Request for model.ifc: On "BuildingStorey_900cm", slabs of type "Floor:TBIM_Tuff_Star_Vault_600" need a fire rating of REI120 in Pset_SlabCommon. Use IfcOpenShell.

First a look at what the model holds.

```python
import ifcopenshell
import ifcopenshell.util.element

model = ifcopenshell.open("model.ifc")
print(model.schema)
storey = next(s for s in model.by_type("IfcBuildingStorey") if s.Name == "BuildingStorey_900cm")
slabs = [e for e in ifcopenshell.util.element.get_decomposition(storey) if e.is_a("IfcSlab")]
seen = {}
for e in slabs:
    element_type = ifcopenshell.util.element.get_type(e)
    key = (element_type.Name if element_type != e and element_type else None, ifcopenshell.util.element.get_pset(e, "Pset_SlabCommon", "FireRating"))
    seen[key] = seen.get(key, 0) + 1
for (name, value), count in sorted(seen.items(), key=str):
    print(count, "x", name, "|", value)
```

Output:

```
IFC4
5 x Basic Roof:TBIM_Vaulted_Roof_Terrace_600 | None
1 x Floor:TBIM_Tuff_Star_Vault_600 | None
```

```python
import ifcopenshell
import ifcopenshell.api.pset
import ifcopenshell.util.element

model = ifcopenshell.open("model.ifc")

storey = next(s for s in model.by_type("IfcBuildingStorey") if s.Name == "BuildingStorey_900cm")
slabs = [e for e in ifcopenshell.util.element.get_decomposition(storey) if e.is_a("IfcSlab")]

count = 0
for e in slabs:
    element_type = ifcopenshell.util.element.get_type(e)
    if element_type in (None, e) or element_type.Name != "Floor:TBIM_Tuff_Star_Vault_600":
        continue
    # add_pset returns the element's existing set when there is one.
    pset = ifcopenshell.api.pset.add_pset(model, product=e, name="Pset_SlabCommon")
    ifcopenshell.api.pset.edit_pset(model, pset=pset, properties={"FireRating": "REI120"})
    count += 1

print(count, "slabs updated")

model.write("model_edited.ifc")
```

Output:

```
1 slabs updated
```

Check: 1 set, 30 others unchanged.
